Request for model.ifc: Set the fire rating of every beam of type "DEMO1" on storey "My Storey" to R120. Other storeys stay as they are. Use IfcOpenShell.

First a look at what the model holds.

```python
import ifcopenshell
import ifcopenshell.util.element

model = ifcopenshell.open("model.ifc")
print(model.schema)
storey = next(s for s in model.by_type("IfcBuildingStorey") if s.Name == "My Storey")
beams = [e for e in ifcopenshell.util.element.get_decomposition(storey) if e.is_a("IfcBeam")]
seen = {}
for e in beams:
    element_type = ifcopenshell.util.element.get_type(e)
    key = (element_type.Name if element_type != e and element_type else None, ifcopenshell.util.element.get_pset(e, "Pset_BeamCommon", "FireRating"))
    seen[key] = seen.get(key, 0) + 1
for (name, value), count in sorted(seen.items(), key=str):
    print(count, "x", name, "|", value)
```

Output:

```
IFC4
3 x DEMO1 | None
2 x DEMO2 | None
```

```python
import ifcopenshell
import ifcopenshell.api.pset
import ifcopenshell.util.element

model = ifcopenshell.open("model.ifc")

storey = next(s for s in model.by_type("IfcBuildingStorey") if s.Name == "My Storey")
beams = [e for e in ifcopenshell.util.element.get_decomposition(storey) if e.is_a("IfcBeam")]

count = 0
for e in beams:
    element_type = ifcopenshell.util.element.get_type(e)
    if element_type in (None, e) or element_type.Name != "DEMO1":
        continue
    # add_pset returns the element's existing set when there is one.
    pset = ifcopenshell.api.pset.add_pset(model, product=e, name="Pset_BeamCommon")
    ifcopenshell.api.pset.edit_pset(model, pset=pset, properties={"FireRating": "R120"})
    count += 1

print(count, "beams updated")

model.write("model_edited.ifc")
```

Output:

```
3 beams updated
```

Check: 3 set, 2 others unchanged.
